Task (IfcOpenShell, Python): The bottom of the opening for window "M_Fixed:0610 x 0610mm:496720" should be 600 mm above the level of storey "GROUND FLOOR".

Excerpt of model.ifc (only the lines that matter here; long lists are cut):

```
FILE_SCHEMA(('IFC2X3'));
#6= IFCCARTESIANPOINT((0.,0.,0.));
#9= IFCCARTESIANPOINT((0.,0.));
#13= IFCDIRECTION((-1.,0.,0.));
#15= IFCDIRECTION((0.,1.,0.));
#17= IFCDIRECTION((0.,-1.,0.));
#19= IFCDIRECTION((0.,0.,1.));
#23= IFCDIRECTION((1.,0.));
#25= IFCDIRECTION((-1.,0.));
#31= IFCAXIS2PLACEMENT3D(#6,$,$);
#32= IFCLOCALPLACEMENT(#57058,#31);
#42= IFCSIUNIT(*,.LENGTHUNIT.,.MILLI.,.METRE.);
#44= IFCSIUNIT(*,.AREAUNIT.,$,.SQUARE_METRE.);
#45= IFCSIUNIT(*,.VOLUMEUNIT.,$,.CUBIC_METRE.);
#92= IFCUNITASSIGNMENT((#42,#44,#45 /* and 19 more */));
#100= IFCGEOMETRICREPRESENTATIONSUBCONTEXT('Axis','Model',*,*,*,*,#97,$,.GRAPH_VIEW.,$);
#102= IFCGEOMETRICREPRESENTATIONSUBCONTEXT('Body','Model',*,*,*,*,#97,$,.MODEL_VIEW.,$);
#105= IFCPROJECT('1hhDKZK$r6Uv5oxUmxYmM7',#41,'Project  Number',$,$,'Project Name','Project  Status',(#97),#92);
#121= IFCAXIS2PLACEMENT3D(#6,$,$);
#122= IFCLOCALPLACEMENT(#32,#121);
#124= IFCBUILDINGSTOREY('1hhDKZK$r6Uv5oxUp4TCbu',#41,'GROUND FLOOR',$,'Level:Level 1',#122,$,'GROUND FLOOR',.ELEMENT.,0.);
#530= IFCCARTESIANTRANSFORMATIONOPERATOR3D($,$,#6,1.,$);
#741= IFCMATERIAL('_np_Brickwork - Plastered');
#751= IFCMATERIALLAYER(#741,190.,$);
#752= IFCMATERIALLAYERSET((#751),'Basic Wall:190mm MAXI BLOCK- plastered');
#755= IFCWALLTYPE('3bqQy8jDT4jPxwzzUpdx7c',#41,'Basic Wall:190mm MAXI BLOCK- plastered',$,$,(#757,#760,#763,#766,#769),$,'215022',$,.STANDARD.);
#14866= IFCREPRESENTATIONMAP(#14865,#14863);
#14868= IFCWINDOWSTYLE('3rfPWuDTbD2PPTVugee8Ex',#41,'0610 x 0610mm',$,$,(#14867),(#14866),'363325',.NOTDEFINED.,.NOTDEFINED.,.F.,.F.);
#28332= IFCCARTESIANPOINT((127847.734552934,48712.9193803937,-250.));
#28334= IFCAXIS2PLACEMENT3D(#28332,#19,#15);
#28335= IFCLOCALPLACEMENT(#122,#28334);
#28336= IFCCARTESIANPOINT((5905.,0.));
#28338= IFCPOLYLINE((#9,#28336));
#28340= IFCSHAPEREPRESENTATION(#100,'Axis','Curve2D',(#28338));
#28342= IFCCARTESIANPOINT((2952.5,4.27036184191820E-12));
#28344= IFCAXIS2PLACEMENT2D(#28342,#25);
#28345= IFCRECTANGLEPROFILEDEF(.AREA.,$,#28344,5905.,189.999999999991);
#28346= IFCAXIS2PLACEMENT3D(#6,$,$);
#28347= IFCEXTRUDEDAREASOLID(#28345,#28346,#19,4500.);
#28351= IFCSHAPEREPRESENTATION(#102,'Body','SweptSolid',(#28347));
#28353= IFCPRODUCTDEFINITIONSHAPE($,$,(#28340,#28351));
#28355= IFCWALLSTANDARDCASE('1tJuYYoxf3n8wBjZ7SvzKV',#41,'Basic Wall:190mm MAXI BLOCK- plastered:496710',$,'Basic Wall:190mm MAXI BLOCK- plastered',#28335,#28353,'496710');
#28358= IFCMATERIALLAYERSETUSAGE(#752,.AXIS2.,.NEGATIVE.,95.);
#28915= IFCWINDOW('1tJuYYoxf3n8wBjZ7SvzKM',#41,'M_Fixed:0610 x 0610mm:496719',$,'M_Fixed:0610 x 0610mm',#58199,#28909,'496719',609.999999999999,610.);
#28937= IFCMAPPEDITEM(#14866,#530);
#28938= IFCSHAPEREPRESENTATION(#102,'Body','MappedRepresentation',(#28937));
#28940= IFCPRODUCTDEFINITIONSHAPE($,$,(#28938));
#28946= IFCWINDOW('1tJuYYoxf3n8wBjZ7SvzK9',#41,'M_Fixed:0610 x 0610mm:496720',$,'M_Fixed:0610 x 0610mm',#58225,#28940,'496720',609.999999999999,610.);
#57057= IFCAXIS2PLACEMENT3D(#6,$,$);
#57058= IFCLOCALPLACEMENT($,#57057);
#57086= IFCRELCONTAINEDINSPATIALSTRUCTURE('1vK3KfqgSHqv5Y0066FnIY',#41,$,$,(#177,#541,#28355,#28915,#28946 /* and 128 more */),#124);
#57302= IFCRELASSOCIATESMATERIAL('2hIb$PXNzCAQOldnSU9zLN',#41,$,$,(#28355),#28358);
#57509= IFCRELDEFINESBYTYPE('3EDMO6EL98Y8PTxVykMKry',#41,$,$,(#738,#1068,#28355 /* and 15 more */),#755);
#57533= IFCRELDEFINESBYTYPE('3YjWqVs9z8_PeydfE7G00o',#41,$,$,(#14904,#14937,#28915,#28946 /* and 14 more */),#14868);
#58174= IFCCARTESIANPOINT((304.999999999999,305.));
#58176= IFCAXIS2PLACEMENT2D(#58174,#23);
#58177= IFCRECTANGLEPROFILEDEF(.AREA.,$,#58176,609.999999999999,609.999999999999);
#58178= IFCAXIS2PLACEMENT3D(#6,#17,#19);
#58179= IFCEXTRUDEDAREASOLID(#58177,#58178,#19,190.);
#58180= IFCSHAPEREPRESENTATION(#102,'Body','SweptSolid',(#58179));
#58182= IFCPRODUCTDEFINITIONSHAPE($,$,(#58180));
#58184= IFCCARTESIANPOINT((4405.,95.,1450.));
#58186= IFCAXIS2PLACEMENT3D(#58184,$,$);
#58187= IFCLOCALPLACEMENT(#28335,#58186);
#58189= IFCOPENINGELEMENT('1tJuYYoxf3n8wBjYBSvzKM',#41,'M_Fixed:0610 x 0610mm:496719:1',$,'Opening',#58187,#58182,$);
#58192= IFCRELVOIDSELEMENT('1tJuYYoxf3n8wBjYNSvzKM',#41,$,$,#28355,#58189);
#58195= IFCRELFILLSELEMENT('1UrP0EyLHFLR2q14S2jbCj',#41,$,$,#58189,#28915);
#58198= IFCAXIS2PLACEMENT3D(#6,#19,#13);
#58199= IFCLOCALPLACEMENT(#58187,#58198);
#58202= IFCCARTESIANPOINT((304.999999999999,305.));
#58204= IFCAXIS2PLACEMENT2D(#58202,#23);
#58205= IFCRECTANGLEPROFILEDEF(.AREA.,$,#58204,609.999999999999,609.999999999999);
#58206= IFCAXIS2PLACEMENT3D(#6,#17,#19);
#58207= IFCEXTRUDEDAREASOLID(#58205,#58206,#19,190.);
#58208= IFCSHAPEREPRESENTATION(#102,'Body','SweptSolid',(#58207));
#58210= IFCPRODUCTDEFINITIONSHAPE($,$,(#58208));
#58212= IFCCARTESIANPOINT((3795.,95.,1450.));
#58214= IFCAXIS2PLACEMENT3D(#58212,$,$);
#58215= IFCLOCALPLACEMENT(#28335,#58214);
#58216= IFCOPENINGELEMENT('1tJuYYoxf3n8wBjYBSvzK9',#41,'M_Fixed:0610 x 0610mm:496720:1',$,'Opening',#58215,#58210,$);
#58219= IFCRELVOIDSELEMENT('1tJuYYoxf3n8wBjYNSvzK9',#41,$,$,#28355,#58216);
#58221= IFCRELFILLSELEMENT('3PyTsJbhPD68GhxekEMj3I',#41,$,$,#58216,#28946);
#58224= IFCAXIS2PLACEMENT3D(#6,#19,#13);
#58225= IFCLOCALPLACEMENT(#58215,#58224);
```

```python
import numpy as np
import ifcopenshell
import ifcopenshell.api.geometry
import ifcopenshell.geom
import ifcopenshell.util.element
import ifcopenshell.util.placement
import ifcopenshell.util.shape
import ifcopenshell.util.unit

model = ifcopenshell.open("model.ifc")
unit_scale = ifcopenshell.util.unit.calculate_unit_scale(model)

window = model.by_guid("1tJuYYoxf3n8wBjZ7SvzK9")
opening = window.FillsVoids[0].RelatingOpeningElement
storey = ifcopenshell.util.element.get_container(window, ifc_class="IfcBuildingStorey")
level = ifcopenshell.util.placement.get_local_placement(storey.ObjectPlacement)[2, 3]

# The opening's origin need not be at the sill, so measure its lowest point.
shape = ifcopenshell.geom.create_shape(ifcopenshell.geom.settings(), opening)
bottom = ifcopenshell.util.shape.get_shape_bottom_elevation(shape, shape.geometry) / unit_scale
dz = level + 0.6 / unit_scale - bottom

shift = np.array([0.0, 0.0, dz])
# The window is placed relative to its opening, so it follows when the opening moves.
matrix = ifcopenshell.util.placement.get_local_placement(opening.ObjectPlacement)
matrix[:3, 3] += shift
ifcopenshell.api.geometry.edit_object_placement(
    model, product=opening, matrix=matrix, is_si=False, should_transform_children=True
)

print(f"moved by {dz * unit_scale:+.3f} m")

model.write("model_rev.ifc")
```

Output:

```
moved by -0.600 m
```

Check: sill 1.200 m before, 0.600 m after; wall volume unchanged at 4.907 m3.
